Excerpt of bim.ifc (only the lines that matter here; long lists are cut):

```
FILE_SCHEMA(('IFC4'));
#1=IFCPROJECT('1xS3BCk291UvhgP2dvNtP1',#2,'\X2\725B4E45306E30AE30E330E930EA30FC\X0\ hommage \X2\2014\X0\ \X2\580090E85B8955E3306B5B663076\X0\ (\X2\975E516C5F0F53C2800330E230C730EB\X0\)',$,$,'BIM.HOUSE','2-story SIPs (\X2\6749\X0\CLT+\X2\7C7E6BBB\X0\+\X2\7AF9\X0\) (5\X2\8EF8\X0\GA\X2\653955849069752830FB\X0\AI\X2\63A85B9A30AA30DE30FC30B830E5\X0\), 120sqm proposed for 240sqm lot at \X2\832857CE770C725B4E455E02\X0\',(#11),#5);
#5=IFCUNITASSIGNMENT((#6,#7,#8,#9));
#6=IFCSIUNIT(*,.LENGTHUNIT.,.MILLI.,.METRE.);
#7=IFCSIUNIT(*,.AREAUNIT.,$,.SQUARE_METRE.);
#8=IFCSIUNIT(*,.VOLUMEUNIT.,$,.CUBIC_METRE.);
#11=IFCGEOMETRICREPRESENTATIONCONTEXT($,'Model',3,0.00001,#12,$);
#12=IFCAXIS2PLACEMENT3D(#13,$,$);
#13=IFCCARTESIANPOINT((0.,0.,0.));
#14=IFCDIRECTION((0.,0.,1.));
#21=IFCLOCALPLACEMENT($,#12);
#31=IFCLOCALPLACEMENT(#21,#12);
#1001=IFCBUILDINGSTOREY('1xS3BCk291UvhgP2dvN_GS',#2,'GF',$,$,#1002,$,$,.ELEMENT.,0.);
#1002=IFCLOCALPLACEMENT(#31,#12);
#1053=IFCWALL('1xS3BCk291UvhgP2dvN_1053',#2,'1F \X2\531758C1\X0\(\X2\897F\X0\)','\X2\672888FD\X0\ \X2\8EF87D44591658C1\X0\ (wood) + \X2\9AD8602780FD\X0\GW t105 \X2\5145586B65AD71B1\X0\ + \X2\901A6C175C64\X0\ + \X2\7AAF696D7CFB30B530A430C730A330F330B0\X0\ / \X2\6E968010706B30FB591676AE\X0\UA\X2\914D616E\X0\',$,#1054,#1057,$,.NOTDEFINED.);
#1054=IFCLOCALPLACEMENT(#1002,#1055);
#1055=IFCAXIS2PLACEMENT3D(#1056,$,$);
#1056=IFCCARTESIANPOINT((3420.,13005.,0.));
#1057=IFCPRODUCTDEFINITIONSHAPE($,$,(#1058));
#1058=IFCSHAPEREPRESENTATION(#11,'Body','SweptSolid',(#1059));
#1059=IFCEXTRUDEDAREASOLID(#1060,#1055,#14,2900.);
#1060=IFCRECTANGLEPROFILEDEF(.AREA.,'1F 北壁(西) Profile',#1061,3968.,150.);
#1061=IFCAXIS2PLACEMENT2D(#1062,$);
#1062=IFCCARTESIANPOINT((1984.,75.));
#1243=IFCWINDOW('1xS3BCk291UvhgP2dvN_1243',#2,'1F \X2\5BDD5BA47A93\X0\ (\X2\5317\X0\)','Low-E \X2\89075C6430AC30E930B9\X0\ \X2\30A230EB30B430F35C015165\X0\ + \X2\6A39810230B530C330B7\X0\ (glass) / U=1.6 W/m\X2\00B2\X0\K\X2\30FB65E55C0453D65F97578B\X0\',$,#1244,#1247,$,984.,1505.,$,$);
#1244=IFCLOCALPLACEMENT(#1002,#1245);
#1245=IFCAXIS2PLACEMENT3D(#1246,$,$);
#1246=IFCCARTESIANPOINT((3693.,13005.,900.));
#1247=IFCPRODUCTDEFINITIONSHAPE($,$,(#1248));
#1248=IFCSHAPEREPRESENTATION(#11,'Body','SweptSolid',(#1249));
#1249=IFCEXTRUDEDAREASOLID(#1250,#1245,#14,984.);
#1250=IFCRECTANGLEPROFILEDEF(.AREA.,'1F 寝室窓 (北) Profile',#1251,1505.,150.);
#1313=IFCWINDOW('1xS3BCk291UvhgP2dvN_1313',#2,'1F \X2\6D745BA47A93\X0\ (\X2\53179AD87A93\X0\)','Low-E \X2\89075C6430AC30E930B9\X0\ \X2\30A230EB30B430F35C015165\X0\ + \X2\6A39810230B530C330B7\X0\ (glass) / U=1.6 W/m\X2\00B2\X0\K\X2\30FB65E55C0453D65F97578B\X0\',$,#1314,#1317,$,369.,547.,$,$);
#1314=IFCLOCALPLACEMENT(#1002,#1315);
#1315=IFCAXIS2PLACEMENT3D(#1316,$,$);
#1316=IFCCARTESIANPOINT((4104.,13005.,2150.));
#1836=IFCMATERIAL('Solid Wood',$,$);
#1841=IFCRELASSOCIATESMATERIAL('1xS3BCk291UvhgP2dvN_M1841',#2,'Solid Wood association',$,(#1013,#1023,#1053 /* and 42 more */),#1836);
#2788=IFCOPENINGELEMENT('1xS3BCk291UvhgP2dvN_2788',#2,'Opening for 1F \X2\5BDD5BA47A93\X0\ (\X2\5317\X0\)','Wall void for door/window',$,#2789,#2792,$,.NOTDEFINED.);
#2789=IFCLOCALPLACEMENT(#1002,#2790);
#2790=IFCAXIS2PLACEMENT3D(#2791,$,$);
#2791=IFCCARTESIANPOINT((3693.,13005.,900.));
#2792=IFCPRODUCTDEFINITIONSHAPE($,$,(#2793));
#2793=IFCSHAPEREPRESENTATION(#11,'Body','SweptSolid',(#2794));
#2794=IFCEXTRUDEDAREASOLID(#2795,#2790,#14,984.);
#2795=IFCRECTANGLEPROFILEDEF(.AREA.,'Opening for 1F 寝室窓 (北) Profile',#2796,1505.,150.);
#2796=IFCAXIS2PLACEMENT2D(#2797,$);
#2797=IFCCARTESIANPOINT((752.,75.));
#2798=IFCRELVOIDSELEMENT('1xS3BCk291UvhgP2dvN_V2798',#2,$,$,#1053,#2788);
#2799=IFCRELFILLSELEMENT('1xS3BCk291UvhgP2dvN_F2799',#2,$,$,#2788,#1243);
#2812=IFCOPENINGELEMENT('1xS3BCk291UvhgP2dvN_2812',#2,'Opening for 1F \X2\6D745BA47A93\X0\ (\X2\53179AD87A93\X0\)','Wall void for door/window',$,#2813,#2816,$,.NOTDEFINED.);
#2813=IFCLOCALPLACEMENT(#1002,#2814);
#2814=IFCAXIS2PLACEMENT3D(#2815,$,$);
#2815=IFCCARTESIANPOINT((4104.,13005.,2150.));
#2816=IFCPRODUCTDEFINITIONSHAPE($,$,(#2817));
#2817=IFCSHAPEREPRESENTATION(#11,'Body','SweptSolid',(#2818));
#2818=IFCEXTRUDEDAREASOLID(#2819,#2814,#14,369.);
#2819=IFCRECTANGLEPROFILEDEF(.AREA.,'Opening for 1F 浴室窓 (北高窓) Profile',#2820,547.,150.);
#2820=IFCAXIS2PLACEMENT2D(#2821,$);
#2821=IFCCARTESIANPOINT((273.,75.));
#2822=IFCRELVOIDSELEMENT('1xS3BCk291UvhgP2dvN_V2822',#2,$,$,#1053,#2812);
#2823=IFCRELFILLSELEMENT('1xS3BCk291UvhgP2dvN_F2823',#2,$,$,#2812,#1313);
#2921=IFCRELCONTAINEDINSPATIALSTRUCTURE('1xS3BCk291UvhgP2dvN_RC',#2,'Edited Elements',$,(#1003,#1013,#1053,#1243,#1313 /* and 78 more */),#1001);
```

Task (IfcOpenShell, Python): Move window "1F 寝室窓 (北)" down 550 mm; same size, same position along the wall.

```python
import numpy as np
import ifcopenshell
import ifcopenshell.api.geometry
import ifcopenshell.util.placement
import ifcopenshell.util.unit

model = ifcopenshell.open("bim.ifc")
unit_scale = ifcopenshell.util.unit.calculate_unit_scale(model)

window = model.by_guid("1xS3BCk291UvhgP2dvN_1243")
opening = window.FillsVoids[0].RelatingOpeningElement
dz = -0.55 / unit_scale

shift = np.array([0.0, 0.0, dz])
# The window is not placed relative to its opening, so move both.
for product in (opening, window):
    matrix = ifcopenshell.util.placement.get_local_placement(product.ObjectPlacement)
    matrix[:3, 3] += shift
    ifcopenshell.api.geometry.edit_object_placement(model, product=product, matrix=matrix, is_si=False)

print(f"moved by {dz * unit_scale:+.3f} m")

model.write("bim-out.ifc")
```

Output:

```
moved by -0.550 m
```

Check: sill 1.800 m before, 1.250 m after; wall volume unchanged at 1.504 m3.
